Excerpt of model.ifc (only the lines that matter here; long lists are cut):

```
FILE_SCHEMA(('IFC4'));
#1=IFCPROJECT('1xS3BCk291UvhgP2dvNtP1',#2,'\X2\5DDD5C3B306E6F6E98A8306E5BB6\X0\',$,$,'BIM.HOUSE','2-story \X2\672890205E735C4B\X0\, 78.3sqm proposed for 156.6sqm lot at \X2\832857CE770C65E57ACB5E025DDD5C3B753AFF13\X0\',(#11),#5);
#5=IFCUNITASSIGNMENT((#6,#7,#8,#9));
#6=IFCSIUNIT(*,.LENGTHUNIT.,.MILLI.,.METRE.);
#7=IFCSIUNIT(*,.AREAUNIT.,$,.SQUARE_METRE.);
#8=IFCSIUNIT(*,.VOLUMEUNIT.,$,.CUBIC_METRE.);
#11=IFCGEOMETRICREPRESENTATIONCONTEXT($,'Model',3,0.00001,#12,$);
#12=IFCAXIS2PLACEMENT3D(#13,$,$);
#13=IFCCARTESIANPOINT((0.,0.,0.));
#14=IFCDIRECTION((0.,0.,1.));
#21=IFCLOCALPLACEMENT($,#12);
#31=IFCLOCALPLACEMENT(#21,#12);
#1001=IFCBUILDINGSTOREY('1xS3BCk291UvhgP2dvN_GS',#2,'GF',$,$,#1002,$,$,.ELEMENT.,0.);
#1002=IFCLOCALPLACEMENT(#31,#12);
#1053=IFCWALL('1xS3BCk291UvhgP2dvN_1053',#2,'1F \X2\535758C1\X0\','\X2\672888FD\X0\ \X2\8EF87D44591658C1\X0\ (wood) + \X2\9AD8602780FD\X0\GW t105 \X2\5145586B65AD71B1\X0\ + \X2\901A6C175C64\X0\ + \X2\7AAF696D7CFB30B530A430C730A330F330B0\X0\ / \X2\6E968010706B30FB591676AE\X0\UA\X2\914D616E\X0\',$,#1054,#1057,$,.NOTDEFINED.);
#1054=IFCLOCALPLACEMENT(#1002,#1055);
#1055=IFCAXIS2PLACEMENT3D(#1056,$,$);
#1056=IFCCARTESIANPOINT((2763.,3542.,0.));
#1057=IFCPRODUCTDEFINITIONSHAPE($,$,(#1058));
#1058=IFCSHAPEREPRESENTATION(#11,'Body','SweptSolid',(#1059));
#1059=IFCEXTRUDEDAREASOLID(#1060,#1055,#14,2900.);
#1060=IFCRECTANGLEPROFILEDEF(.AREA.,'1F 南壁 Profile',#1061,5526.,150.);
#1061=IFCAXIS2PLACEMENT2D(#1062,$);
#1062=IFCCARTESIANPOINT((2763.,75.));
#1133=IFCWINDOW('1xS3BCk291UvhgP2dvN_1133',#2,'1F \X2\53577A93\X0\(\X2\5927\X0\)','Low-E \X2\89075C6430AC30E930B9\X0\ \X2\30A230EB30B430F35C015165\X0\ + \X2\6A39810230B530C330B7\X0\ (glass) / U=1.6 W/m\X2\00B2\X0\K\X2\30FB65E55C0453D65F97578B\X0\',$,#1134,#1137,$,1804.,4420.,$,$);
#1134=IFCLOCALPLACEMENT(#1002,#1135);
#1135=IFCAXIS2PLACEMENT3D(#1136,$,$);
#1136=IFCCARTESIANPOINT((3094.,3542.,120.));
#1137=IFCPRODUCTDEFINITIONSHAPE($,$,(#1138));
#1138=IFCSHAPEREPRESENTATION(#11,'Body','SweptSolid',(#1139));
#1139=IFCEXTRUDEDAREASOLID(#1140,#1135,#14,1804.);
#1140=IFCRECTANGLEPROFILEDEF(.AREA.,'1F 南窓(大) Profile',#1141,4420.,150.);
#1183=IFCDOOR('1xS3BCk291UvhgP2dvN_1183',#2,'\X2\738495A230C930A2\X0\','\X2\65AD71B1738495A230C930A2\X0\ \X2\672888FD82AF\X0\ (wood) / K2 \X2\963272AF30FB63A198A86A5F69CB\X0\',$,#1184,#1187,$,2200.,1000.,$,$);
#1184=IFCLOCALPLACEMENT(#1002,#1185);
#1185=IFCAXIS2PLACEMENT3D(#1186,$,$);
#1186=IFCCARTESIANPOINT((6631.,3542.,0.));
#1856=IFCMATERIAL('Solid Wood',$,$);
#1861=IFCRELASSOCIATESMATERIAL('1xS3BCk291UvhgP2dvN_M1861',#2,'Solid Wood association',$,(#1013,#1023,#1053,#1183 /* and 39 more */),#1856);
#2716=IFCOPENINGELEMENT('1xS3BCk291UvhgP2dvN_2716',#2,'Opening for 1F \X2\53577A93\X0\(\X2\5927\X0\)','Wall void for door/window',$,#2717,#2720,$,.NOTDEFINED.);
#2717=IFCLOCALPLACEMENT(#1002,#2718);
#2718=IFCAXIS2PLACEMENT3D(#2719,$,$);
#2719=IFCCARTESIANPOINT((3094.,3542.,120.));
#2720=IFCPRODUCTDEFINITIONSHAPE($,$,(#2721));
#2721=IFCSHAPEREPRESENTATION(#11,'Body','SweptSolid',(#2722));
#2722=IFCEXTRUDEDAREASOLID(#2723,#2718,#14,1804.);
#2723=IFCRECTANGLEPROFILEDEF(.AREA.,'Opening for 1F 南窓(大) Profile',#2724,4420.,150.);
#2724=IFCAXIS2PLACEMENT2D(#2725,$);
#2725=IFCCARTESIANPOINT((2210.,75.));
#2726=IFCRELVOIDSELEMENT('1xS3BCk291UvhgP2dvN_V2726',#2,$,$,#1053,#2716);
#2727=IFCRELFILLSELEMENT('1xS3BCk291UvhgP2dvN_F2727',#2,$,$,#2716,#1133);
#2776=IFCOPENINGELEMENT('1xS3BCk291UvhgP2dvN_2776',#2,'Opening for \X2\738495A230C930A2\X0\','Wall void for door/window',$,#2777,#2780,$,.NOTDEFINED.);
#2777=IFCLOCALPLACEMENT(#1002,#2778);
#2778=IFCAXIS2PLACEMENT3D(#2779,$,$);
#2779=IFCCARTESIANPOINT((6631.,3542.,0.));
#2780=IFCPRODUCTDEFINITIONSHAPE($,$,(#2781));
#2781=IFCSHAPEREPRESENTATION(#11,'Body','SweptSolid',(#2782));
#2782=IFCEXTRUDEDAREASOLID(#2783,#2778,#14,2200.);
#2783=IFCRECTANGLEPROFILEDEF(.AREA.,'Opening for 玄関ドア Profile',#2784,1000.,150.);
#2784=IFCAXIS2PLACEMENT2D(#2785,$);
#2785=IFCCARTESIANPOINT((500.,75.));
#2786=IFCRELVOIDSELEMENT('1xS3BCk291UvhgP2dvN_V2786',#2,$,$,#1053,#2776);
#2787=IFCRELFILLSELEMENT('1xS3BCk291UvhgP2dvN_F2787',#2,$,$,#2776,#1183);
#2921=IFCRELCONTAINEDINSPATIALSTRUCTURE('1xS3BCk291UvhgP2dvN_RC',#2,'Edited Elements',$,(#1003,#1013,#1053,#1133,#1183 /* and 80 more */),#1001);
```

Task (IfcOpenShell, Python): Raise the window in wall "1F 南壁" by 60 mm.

```python
import numpy as np
import ifcopenshell
import ifcopenshell.api.geometry
import ifcopenshell.util.placement
import ifcopenshell.util.unit

model = ifcopenshell.open("model.ifc")
unit_scale = ifcopenshell.util.unit.calculate_unit_scale(model)

window = model.by_guid("1xS3BCk291UvhgP2dvN_1133")
opening = window.FillsVoids[0].RelatingOpeningElement
dz = 0.06 / unit_scale

shift = np.array([0.0, 0.0, dz])
# The window is not placed relative to its opening, so move both.
for product in (opening, window):
    matrix = ifcopenshell.util.placement.get_local_placement(product.ObjectPlacement)
    matrix[:3, 3] += shift
    ifcopenshell.api.geometry.edit_object_placement(model, product=product, matrix=matrix, is_si=False)

print(f"moved by {dz * unit_scale:+.3f} m")

model.write("model_edited.ifc")
```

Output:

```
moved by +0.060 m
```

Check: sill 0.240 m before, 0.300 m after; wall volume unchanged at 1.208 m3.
